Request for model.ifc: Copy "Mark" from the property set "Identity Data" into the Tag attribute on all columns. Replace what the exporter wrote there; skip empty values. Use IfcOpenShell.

First a look at what the model holds.

```python
import ifcopenshell
import ifcopenshell.util.element

model = ifcopenshell.open("model.ifc")
print(model.schema)
columns = model.by_type("IfcColumn")
print(len(columns), "columns")
for e in columns[:8]:
    source = ifcopenshell.util.element.get_pset(e, "Identity Data", "Mark")
    target = e.Tag
    print(e.id(), repr(source), repr(target), sep=" | ")
```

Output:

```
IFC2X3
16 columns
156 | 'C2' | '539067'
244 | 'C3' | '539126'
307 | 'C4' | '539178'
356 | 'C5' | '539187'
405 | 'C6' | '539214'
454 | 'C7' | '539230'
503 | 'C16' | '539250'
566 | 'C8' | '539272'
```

```python
import ifcopenshell
import ifcopenshell.util.element

model = ifcopenshell.open("model.ifc")

count = 0
for e in model.by_type("IfcColumn"):
    value = ifcopenshell.util.element.get_pset(e, "Identity Data", "Mark")
    current = e.Tag
    if not value or not value.strip() or current == value:
        continue
    e.Tag = value
    count += 1

print(count, "columns updated")

model.write("model_edited.ifc")
```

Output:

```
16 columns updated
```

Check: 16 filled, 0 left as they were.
